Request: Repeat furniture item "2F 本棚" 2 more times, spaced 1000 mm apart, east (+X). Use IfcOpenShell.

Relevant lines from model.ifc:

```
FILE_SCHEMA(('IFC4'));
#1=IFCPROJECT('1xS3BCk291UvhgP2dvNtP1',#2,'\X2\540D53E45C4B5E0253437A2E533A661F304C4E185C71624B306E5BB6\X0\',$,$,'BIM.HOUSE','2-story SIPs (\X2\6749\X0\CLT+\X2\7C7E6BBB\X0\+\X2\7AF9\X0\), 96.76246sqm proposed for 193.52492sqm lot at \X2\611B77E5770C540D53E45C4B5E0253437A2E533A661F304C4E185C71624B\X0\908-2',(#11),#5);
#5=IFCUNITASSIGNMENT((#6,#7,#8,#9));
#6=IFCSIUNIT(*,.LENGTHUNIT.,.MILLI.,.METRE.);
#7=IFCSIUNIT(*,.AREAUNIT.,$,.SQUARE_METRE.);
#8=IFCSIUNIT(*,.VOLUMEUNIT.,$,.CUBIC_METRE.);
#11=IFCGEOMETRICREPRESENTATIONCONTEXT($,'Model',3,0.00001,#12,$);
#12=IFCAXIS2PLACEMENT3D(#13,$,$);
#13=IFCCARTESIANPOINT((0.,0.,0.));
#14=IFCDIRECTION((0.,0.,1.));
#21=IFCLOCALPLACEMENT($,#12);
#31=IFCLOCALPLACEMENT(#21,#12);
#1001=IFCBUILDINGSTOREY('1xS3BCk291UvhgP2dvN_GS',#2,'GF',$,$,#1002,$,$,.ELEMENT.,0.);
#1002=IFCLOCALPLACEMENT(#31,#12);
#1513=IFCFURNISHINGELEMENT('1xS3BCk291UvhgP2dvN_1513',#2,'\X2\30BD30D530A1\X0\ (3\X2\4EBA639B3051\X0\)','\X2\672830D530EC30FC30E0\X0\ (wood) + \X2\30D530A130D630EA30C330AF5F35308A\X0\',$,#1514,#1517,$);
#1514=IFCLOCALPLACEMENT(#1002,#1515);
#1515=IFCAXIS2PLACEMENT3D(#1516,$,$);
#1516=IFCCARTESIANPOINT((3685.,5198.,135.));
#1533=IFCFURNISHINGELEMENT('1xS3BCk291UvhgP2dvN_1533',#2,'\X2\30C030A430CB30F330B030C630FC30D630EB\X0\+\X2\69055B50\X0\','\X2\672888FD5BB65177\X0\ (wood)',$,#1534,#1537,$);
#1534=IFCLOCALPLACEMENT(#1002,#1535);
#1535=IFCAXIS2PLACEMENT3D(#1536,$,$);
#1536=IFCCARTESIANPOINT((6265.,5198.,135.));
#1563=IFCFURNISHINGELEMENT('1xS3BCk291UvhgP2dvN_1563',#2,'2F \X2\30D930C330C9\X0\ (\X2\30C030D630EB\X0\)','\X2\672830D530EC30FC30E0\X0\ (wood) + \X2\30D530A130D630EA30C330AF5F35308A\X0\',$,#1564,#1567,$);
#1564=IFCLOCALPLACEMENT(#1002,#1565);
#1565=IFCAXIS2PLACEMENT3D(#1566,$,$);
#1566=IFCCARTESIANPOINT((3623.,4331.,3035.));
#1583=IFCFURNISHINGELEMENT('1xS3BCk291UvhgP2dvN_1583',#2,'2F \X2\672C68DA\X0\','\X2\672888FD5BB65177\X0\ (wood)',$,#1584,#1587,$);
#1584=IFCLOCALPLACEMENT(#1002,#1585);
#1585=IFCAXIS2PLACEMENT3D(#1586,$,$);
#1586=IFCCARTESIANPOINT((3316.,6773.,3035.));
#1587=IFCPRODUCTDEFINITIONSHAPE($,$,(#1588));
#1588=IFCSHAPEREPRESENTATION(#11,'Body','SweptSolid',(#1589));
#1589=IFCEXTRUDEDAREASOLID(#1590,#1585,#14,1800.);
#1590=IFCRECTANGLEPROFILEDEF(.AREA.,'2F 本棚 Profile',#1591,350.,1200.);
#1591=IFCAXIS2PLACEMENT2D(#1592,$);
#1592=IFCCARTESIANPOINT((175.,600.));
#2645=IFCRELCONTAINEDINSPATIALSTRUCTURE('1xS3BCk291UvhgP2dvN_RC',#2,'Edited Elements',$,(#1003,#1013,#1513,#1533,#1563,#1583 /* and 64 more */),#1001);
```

```python
import numpy as np
import ifcopenshell
import ifcopenshell.api.geometry
import ifcopenshell.api.root
import ifcopenshell.util.element
import ifcopenshell.util.placement
import ifcopenshell.util.unit

model = ifcopenshell.open("model.ifc")
unit_scale = ifcopenshell.util.unit.calculate_unit_scale(model)


def reuse_history(source, copy):
    """copy_class also copies each property set's owner history, people and application; keep the originals."""
    for rel in copy.IsDefinedBy:
        if rel.is_a("IfcRelDefinesByProperties") and (history := rel.RelatingPropertyDefinition.OwnerHistory):
            rel.RelatingPropertyDefinition.OwnerHistory = source.OwnerHistory
            ifcopenshell.util.element.remove_deep2(model, history)


source = model.by_guid("1xS3BCk291UvhgP2dvN_1583")
base = ifcopenshell.util.placement.get_local_placement(source.ObjectPlacement)
step = np.array([1.0, 0.0, 0.0]) * 1 / unit_scale

for i in range(1, 3):
    copy = ifcopenshell.api.root.copy_class(model, product=source)
    copy.Representation = ifcopenshell.util.element.copy_deep(
        model, source.Representation, exclude=["IfcGeometricRepresentationContext", "IfcRepresentationMap"]
    )
    reuse_history(source, copy)
    matrix = base.copy()
    matrix[:3, 3] += i * step
    print("added at", matrix[:3, 3].round(3) + 0.0)
    ifcopenshell.api.geometry.edit_object_placement(model, product=copy, matrix=matrix, is_si=False)

model.write("model_v2.ifc")
```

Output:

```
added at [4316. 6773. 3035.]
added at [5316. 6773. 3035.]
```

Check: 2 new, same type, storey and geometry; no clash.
